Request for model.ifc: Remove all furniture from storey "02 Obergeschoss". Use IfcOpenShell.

First a look at what the model holds.

```python
import ifcopenshell
import ifcopenshell.util.element

model = ifcopenshell.open("model.ifc")
print(model.schema)
storey = next(s for s in model.by_type("IfcBuildingStorey") if s.Name == "02 Obergeschoss")
furniture = [e for e in ifcopenshell.util.element.get_decomposition(storey) if e.is_a("IfcFurnishingElement")]
seen = {}
for e in furniture:
    element_type = ifcopenshell.util.element.get_type(e)
    name = element_type.Name if element_type not in (None, e) else None
    seen[name] = seen.get(name, 0) + 1
for name, count in sorted(seen.items(), key=str):
    print(count, "x", name)
```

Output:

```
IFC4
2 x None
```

```python
import ifcopenshell
import ifcopenshell.api.root
import ifcopenshell.util.element

model = ifcopenshell.open("model.ifc")

storey = next(s for s in model.by_type("IfcBuildingStorey") if s.Name == "02 Obergeschoss")
furniture = [e for e in ifcopenshell.util.element.get_decomposition(storey) if e.is_a("IfcFurnishingElement")]

for e in furniture:
    ifcopenshell.api.root.remove_product(model, product=e)
print(len(furniture), "removed")

model.write("model_edited.ifc")
```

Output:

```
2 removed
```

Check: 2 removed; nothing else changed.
